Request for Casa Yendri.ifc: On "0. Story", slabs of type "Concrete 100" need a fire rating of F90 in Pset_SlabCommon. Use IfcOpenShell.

First a look at what the model holds.

```python
import ifcopenshell
import ifcopenshell.util.element

model = ifcopenshell.open("Casa Yendri.ifc")
print(model.schema)
storey = next(s for s in model.by_type("IfcBuildingStorey") if s.Name == "0. Story")
slabs = [e for e in ifcopenshell.util.element.get_decomposition(storey) if e.is_a("IfcSlab")]
seen = {}
for e in slabs:
    element_type = ifcopenshell.util.element.get_type(e)
    key = (element_type.Name if element_type != e and element_type else None, ifcopenshell.util.element.get_pset(e, "Pset_SlabCommon", "FireRating"))
    seen[key] = seen.get(key, 0) + 1
for (name, value), count in sorted(seen.items(), key=str):
    print(count, "x", name, "|", value)
```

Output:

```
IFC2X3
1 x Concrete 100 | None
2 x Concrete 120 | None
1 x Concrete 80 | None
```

```python
import ifcopenshell
import ifcopenshell.api.pset
import ifcopenshell.util.element

model = ifcopenshell.open("Casa Yendri.ifc")

storey = next(s for s in model.by_type("IfcBuildingStorey") if s.Name == "0. Story")
slabs = [e for e in ifcopenshell.util.element.get_decomposition(storey) if e.is_a("IfcSlab")]

count = 0
for e in slabs:
    element_type = ifcopenshell.util.element.get_type(e)
    if element_type in (None, e) or element_type.Name != "Concrete 100":
        continue
    # add_pset returns the element's existing set when there is one.
    pset = ifcopenshell.api.pset.add_pset(model, product=e, name="Pset_SlabCommon")
    ifcopenshell.api.pset.edit_pset(model, pset=pset, properties={"FireRating": "F90"})
    count += 1

print(count, "slabs updated")

model.write("Casa Yendri_rev.ifc")
```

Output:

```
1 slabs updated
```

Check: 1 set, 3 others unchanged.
